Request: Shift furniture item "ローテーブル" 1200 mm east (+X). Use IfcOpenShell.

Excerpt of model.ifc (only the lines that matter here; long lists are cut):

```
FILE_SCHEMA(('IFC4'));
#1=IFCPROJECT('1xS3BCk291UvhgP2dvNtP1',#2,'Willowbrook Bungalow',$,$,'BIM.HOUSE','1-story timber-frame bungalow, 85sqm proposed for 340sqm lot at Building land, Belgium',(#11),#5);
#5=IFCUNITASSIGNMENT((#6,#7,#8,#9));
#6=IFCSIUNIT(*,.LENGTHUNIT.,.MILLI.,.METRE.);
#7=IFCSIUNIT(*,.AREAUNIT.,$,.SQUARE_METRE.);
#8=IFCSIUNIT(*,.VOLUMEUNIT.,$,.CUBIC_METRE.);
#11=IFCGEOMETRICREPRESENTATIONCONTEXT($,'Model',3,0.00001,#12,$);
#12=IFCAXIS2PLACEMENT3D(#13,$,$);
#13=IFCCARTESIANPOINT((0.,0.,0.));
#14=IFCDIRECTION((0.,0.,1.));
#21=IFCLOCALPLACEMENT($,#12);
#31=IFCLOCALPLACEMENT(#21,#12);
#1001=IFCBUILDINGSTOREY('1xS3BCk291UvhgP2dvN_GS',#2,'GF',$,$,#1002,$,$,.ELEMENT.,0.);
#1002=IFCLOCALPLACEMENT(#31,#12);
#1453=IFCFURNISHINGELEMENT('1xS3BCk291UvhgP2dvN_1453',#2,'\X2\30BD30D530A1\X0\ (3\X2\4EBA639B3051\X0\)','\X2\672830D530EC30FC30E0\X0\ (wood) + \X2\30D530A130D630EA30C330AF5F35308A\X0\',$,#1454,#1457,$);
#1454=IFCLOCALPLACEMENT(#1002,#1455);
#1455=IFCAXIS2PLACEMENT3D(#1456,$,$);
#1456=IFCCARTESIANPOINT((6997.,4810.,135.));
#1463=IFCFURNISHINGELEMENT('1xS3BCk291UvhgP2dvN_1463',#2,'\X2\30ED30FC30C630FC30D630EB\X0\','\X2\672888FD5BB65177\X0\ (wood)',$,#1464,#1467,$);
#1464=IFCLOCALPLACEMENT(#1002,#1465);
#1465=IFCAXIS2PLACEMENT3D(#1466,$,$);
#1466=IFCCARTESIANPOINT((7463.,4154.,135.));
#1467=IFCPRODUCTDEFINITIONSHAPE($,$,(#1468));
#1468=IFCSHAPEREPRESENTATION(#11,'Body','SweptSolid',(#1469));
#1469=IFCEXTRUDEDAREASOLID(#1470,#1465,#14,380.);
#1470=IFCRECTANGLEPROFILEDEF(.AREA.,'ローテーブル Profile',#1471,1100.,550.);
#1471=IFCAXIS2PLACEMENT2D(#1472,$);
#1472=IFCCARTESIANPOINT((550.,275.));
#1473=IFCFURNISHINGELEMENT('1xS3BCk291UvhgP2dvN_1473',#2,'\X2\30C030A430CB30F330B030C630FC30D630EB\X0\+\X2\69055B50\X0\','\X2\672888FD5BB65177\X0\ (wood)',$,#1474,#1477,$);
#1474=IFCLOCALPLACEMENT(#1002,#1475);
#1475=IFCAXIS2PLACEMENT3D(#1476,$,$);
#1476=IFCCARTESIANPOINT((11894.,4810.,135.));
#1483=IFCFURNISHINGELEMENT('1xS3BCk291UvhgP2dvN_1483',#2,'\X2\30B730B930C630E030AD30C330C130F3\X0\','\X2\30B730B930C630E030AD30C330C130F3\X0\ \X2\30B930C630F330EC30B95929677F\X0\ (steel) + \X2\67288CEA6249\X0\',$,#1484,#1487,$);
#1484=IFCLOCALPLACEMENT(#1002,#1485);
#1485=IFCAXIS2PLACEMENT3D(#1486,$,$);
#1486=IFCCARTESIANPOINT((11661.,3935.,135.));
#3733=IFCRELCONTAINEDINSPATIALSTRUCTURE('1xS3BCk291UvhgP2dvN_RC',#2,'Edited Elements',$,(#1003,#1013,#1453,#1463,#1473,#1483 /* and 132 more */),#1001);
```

```python
import ifcopenshell
import ifcopenshell.api.geometry
import ifcopenshell.util.placement

model = ifcopenshell.open("model.ifc")

item = model.by_id(1463)
matrix = ifcopenshell.util.placement.get_local_placement(item.ObjectPlacement)
matrix[0, 3] += 1200.0
ifcopenshell.api.geometry.edit_object_placement(model, product=item, matrix=matrix, is_si=False)

print(ifcopenshell.util.placement.get_local_placement(item.ObjectPlacement).round(3) + 0.0)

model.write("model_updated.ifc")
```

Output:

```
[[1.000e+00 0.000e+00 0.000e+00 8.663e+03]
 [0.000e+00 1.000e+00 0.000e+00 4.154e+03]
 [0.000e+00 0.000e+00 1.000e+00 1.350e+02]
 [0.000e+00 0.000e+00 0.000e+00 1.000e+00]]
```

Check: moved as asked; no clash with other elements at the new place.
